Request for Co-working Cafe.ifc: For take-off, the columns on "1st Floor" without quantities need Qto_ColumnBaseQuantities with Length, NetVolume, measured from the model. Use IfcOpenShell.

First a look at what the model holds.

```python
import ifcopenshell
import ifcopenshell.util.element
import ifcopenshell.util.unit

model = ifcopenshell.open("Co-working Cafe.ifc")
print(model.schema)
for unit_type in ("LENGTHUNIT", "AREAUNIT", "VOLUMEUNIT"):
    print(unit_type, ifcopenshell.util.unit.calculate_unit_scale(model, unit_type))
storey = next(s for s in model.by_type("IfcBuildingStorey") if s.Name == "1st Floor")
columns = [e for e in ifcopenshell.util.element.get_decomposition(storey) if e.is_a("IfcColumn")]
for e in sorted(columns, key=lambda e: e.id()):
    print(e.id(), e.is_a(), e.Name, list(ifcopenshell.util.element.get_psets(e, qtos_only=True)), sep=" | ")
```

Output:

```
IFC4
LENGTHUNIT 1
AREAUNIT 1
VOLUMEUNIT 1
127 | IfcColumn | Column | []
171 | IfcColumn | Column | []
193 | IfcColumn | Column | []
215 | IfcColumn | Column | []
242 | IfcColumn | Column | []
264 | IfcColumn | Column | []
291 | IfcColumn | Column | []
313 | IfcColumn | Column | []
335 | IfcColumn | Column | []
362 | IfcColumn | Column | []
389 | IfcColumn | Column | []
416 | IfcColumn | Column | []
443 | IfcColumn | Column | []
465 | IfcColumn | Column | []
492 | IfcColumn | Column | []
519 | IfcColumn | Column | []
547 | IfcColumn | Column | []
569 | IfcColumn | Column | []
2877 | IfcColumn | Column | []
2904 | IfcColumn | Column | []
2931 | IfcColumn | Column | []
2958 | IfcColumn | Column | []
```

```python
import ifcopenshell
import ifcopenshell.api.pset
import ifcopenshell.geom
import ifcopenshell.util.element
import ifcopenshell.util.shape
import ifcopenshell.util.unit

model = ifcopenshell.open("Co-working Cafe.ifc")
unit_scale = ifcopenshell.util.unit.calculate_unit_scale(model)
volume_scale = ifcopenshell.util.unit.calculate_unit_scale(model, "VOLUMEUNIT")
settings = ifcopenshell.geom.settings()

storey = next(s for s in model.by_type("IfcBuildingStorey") if s.Name == "1st Floor")
columns = [e for e in ifcopenshell.util.element.get_decomposition(storey) if e.is_a("IfcColumn")]

for e in sorted(columns, key=lambda e: e.id()):
    if ifcopenshell.util.element.get_psets(e, qtos_only=True, should_inherit=False):
        continue
    # Geometry comes back in metres, in the element's own axes.
    shape = ifcopenshell.geom.create_shape(settings, e)
    values = {
        "Length": ifcopenshell.util.shape.get_z(shape.geometry) / unit_scale,
        "NetVolume": ifcopenshell.util.shape.get_volume(shape.geometry) / volume_scale,
    }
    qto = ifcopenshell.api.pset.add_qto(model, product=e, name="Qto_ColumnBaseQuantities")
    ifcopenshell.api.pset.edit_qto(model, qto=qto, properties=values)
    print(e.id(), {k: round(v, 3) for k, v in values.items()})

model.write("Co-working Cafe_rev.ifc")
```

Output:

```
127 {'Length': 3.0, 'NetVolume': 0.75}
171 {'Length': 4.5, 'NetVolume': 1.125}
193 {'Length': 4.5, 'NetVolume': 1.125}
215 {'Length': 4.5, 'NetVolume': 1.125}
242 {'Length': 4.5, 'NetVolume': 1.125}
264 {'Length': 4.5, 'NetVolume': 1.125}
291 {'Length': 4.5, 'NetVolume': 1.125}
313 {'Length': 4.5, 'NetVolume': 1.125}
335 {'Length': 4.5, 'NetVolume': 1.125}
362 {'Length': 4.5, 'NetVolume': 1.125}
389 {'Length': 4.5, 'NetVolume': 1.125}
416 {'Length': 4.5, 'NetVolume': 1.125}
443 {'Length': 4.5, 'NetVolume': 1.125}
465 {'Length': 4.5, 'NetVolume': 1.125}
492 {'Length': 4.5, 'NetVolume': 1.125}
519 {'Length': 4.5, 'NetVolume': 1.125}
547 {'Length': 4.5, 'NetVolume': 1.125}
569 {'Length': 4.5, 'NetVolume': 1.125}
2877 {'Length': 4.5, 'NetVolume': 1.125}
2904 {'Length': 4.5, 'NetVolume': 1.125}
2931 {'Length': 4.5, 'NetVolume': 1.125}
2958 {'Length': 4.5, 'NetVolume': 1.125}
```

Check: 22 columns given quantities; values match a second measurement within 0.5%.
